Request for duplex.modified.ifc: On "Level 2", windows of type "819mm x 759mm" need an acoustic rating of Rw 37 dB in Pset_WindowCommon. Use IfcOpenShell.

First a look at what the model holds.

```python
import ifcopenshell
import ifcopenshell.util.element

model = ifcopenshell.open("duplex.modified.ifc")
print(model.schema)
storey = next(s for s in model.by_type("IfcBuildingStorey") if s.Name == "Level 2")
windows = [e for e in ifcopenshell.util.element.get_decomposition(storey) if e.is_a("IfcWindow")]
seen = {}
for e in windows:
    element_type = ifcopenshell.util.element.get_type(e)
    key = (element_type.Name if element_type != e and element_type else None, ifcopenshell.util.element.get_pset(e, "Pset_WindowCommon", "AcousticRating"))
    seen[key] = seen.get(key, 0) + 1
for (name, value), count in sorted(seen.items(), key=str):
    print(count, "x", name, "|", value)
```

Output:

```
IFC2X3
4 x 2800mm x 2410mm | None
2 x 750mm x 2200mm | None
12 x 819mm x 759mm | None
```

```python
import ifcopenshell
import ifcopenshell.api.pset
import ifcopenshell.util.element

model = ifcopenshell.open("duplex.modified.ifc")

storey = next(s for s in model.by_type("IfcBuildingStorey") if s.Name == "Level 2")
windows = [e for e in ifcopenshell.util.element.get_decomposition(storey) if e.is_a("IfcWindow")]

count = 0
for e in windows:
    element_type = ifcopenshell.util.element.get_type(e)
    if element_type in (None, e) or element_type.Name != "819mm x 759mm":
        continue
    # add_pset returns the element's existing set when there is one.
    pset = ifcopenshell.api.pset.add_pset(model, product=e, name="Pset_WindowCommon")
    ifcopenshell.api.pset.edit_pset(model, pset=pset, properties={"AcousticRating": "Rw 37 dB"})
    count += 1

print(count, "windows updated")

model.write("duplex.modified_edited.ifc")
```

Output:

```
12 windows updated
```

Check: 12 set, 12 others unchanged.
